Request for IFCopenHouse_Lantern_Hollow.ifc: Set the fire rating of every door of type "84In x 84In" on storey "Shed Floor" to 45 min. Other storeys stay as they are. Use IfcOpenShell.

First a look at what the model holds.

```python
import ifcopenshell
import ifcopenshell.util.element

model = ifcopenshell.open("IFCopenHouse_Lantern_Hollow.ifc")
print(model.schema)
storey = next(s for s in model.by_type("IfcBuildingStorey") if s.Name == "Shed Floor")
doors = [e for e in ifcopenshell.util.element.get_decomposition(storey) if e.is_a("IfcDoor")]
seen = {}
for e in doors:
    element_type = ifcopenshell.util.element.get_type(e)
    key = (element_type.Name if element_type != e and element_type else None, ifcopenshell.util.element.get_pset(e, "Pset_DoorCommon", "FireRating"))
    seen[key] = seen.get(key, 0) + 1
for (name, value), count in sorted(seen.items(), key=str):
    print(count, "x", name, "|", value)
```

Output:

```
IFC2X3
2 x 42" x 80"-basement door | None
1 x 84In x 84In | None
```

```python
import ifcopenshell
import ifcopenshell.api.pset
import ifcopenshell.util.element

model = ifcopenshell.open("IFCopenHouse_Lantern_Hollow.ifc")

storey = next(s for s in model.by_type("IfcBuildingStorey") if s.Name == "Shed Floor")
doors = [e for e in ifcopenshell.util.element.get_decomposition(storey) if e.is_a("IfcDoor")]

count = 0
for e in doors:
    element_type = ifcopenshell.util.element.get_type(e)
    if element_type in (None, e) or element_type.Name != "84In x 84In":
        continue
    # add_pset returns the element's existing set when there is one.
    pset = ifcopenshell.api.pset.add_pset(model, product=e, name="Pset_DoorCommon")
    ifcopenshell.api.pset.edit_pset(model, pset=pset, properties={"FireRating": "45 min"})
    count += 1

print(count, "doors updated")

model.write("IFCopenHouse_Lantern_Hollow_rev.ifc")
```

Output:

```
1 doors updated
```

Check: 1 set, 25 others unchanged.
